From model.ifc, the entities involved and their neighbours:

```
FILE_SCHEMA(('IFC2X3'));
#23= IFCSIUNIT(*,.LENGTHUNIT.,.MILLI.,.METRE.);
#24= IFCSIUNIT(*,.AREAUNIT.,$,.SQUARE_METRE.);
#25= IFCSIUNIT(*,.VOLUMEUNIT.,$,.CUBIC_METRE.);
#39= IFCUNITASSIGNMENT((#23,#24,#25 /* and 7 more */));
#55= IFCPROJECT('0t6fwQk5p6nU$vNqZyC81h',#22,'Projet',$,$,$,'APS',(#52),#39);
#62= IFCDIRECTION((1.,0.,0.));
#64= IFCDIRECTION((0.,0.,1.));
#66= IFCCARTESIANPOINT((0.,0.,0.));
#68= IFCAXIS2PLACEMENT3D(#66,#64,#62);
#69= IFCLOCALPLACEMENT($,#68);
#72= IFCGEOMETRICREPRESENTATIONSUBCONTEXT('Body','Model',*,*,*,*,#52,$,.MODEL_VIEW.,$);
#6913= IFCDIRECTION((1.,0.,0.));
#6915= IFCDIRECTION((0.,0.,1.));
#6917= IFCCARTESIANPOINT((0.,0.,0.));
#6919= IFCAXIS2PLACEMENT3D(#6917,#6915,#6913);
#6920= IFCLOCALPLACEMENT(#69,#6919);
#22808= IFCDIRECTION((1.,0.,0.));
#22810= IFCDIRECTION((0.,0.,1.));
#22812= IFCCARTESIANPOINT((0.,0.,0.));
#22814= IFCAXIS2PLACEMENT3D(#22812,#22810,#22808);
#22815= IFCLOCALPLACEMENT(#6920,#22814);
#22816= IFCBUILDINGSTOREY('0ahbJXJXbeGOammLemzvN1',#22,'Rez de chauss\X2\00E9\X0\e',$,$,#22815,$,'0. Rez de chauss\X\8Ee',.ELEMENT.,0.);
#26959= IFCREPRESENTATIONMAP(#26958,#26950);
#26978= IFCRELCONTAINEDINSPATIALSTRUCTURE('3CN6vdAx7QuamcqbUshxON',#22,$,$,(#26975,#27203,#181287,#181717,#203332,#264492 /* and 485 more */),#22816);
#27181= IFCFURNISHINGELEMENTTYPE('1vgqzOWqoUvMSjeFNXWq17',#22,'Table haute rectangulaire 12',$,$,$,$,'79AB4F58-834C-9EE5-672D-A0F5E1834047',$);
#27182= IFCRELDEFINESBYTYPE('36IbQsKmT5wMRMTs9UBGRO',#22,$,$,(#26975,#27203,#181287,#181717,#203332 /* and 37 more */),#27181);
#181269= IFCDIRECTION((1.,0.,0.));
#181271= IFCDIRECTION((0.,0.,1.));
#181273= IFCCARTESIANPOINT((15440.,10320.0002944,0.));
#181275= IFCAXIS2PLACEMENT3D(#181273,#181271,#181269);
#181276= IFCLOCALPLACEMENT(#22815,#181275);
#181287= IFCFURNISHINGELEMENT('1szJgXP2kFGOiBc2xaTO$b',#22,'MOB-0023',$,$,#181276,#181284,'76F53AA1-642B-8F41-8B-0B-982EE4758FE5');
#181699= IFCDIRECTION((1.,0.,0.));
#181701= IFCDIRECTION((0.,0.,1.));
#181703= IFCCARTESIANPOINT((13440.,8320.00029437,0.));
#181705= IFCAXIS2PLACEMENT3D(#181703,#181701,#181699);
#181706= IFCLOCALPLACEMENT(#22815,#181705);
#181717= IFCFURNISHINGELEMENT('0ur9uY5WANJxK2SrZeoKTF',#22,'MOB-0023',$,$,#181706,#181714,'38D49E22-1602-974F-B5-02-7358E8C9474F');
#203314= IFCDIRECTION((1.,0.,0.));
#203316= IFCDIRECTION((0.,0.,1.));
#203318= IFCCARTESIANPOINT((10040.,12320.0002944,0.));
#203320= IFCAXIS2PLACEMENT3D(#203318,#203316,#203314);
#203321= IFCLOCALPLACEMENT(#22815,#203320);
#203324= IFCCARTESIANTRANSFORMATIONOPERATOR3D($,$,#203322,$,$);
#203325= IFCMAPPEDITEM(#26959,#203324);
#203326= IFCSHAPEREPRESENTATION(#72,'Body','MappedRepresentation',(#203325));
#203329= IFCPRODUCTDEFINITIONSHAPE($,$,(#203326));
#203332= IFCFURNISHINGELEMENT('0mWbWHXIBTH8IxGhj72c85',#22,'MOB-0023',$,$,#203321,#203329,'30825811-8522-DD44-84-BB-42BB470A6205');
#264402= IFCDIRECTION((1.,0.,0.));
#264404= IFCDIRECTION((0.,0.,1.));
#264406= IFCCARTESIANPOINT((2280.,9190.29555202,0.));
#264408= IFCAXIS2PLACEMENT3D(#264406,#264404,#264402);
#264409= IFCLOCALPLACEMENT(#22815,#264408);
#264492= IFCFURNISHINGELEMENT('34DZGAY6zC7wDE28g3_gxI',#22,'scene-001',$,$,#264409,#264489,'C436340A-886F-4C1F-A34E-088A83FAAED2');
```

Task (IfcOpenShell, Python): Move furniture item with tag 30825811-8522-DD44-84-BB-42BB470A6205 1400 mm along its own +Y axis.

```python
import ifcopenshell
import ifcopenshell.api.geometry
import ifcopenshell.util.placement
import ifcopenshell.util.unit

model = ifcopenshell.open("model.ifc")
unit_scale = ifcopenshell.util.unit.calculate_unit_scale(model)

item = model.by_guid("0mWbWHXIBTH8IxGhj72c85")
matrix = ifcopenshell.util.placement.get_local_placement(item.ObjectPlacement)
matrix[:3, 3] += matrix[:3, 1] * 1.4 / unit_scale
ifcopenshell.api.geometry.edit_object_placement(model, product=item, matrix=matrix, is_si=False)

print(ifcopenshell.util.placement.get_local_placement(item.ObjectPlacement).round(3) + 0.0)

model.write("model-out.ifc")
```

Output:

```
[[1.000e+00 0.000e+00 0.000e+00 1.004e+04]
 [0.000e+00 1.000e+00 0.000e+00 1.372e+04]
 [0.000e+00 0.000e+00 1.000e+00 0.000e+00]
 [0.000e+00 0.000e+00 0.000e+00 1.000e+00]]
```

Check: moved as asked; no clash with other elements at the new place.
